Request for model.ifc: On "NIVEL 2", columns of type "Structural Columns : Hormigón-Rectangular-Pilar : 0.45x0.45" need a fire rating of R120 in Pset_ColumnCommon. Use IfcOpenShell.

First a look at what the model holds.

```python
import ifcopenshell
import ifcopenshell.util.element

model = ifcopenshell.open("model.ifc")
print(model.schema)
storey = next(s for s in model.by_type("IfcBuildingStorey") if s.Name == "NIVEL 2")
columns = [e for e in ifcopenshell.util.element.get_decomposition(storey) if e.is_a("IfcColumn")]
seen = {}
for e in columns:
    element_type = ifcopenshell.util.element.get_type(e)
    key = (element_type.Name if element_type != e and element_type else None, ifcopenshell.util.element.get_pset(e, "Pset_ColumnCommon", "FireRating"))
    seen[key] = seen.get(key, 0) + 1
for (name, value), count in sorted(seen.items(), key=str):
    print(count, "x", name, "|", value)
```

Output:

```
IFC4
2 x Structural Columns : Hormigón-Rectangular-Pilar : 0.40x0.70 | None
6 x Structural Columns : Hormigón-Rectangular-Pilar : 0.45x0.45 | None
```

```python
import ifcopenshell
import ifcopenshell.api.pset
import ifcopenshell.util.element

model = ifcopenshell.open("model.ifc")

storey = next(s for s in model.by_type("IfcBuildingStorey") if s.Name == "NIVEL 2")
columns = [e for e in ifcopenshell.util.element.get_decomposition(storey) if e.is_a("IfcColumn")]

count = 0
for e in columns:
    element_type = ifcopenshell.util.element.get_type(e)
    if element_type in (None, e) or element_type.Name != "Structural Columns : Hormigón-Rectangular-Pilar : 0.45x0.45":
        continue
    # add_pset returns the element's existing set when there is one.
    pset = ifcopenshell.api.pset.add_pset(model, product=e, name="Pset_ColumnCommon")
    ifcopenshell.api.pset.edit_pset(model, pset=pset, properties={"FireRating": "R120"})
    count += 1

print(count, "columns updated")

model.write("model-out.ifc")
```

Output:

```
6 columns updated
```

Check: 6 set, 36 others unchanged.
